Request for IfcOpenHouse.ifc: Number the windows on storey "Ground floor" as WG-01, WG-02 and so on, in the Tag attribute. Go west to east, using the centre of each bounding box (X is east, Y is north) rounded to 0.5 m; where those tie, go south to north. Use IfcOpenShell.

First a look at what the model holds.

```python
import ifcopenshell
import ifcopenshell.util.element
import ifcopenshell.util.placement

model = ifcopenshell.open("IfcOpenHouse.ifc")
print(model.schema)
storey = next(s for s in model.by_type("IfcBuildingStorey") if s.Name == "Ground floor")
windows = [e for e in ifcopenshell.util.element.get_decomposition(storey) if e.is_a("IfcWindow")]
for e in sorted(windows, key=lambda e: e.id()):
    origin = ifcopenshell.util.placement.get_local_placement(e.ObjectPlacement)[:3, 3]
    print(e.id(), e.Tag, e.Name, origin.round(2) + 0.0, sep=" | ")
```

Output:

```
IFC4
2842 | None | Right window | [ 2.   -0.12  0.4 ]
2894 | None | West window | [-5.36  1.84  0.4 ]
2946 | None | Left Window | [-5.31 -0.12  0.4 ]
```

```python
import ifcopenshell
import ifcopenshell.geom
import ifcopenshell.util.element
import ifcopenshell.util.shape

model = ifcopenshell.open("IfcOpenHouse.ifc")
settings = ifcopenshell.geom.settings()
settings.set("use-world-coords", True)


def centre(element):
    shape = ifcopenshell.geom.create_shape(settings, element)
    return ifcopenshell.util.shape.get_bbox_centroid(shape.geometry)


storey = next(s for s in model.by_type("IfcBuildingStorey") if s.Name == "Ground floor")
windows = [e for e in ifcopenshell.util.element.get_decomposition(storey) if e.is_a("IfcWindow")]

# Insertion points can sit at a corner or the storey origin, so sort by the geometry (in metres).
centres = {e: centre(e) for e in windows}
windows.sort(key=lambda e: (round(centres[e][0] / 0.5), centres[e][1]))

for i, e in enumerate(windows, start=1):
    number = f"WG-{i:02d}"
    e.Tag = number
    print(e.id(), number)

model.write("IfcOpenHouse_v2.ifc")
```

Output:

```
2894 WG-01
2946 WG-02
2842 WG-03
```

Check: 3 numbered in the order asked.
